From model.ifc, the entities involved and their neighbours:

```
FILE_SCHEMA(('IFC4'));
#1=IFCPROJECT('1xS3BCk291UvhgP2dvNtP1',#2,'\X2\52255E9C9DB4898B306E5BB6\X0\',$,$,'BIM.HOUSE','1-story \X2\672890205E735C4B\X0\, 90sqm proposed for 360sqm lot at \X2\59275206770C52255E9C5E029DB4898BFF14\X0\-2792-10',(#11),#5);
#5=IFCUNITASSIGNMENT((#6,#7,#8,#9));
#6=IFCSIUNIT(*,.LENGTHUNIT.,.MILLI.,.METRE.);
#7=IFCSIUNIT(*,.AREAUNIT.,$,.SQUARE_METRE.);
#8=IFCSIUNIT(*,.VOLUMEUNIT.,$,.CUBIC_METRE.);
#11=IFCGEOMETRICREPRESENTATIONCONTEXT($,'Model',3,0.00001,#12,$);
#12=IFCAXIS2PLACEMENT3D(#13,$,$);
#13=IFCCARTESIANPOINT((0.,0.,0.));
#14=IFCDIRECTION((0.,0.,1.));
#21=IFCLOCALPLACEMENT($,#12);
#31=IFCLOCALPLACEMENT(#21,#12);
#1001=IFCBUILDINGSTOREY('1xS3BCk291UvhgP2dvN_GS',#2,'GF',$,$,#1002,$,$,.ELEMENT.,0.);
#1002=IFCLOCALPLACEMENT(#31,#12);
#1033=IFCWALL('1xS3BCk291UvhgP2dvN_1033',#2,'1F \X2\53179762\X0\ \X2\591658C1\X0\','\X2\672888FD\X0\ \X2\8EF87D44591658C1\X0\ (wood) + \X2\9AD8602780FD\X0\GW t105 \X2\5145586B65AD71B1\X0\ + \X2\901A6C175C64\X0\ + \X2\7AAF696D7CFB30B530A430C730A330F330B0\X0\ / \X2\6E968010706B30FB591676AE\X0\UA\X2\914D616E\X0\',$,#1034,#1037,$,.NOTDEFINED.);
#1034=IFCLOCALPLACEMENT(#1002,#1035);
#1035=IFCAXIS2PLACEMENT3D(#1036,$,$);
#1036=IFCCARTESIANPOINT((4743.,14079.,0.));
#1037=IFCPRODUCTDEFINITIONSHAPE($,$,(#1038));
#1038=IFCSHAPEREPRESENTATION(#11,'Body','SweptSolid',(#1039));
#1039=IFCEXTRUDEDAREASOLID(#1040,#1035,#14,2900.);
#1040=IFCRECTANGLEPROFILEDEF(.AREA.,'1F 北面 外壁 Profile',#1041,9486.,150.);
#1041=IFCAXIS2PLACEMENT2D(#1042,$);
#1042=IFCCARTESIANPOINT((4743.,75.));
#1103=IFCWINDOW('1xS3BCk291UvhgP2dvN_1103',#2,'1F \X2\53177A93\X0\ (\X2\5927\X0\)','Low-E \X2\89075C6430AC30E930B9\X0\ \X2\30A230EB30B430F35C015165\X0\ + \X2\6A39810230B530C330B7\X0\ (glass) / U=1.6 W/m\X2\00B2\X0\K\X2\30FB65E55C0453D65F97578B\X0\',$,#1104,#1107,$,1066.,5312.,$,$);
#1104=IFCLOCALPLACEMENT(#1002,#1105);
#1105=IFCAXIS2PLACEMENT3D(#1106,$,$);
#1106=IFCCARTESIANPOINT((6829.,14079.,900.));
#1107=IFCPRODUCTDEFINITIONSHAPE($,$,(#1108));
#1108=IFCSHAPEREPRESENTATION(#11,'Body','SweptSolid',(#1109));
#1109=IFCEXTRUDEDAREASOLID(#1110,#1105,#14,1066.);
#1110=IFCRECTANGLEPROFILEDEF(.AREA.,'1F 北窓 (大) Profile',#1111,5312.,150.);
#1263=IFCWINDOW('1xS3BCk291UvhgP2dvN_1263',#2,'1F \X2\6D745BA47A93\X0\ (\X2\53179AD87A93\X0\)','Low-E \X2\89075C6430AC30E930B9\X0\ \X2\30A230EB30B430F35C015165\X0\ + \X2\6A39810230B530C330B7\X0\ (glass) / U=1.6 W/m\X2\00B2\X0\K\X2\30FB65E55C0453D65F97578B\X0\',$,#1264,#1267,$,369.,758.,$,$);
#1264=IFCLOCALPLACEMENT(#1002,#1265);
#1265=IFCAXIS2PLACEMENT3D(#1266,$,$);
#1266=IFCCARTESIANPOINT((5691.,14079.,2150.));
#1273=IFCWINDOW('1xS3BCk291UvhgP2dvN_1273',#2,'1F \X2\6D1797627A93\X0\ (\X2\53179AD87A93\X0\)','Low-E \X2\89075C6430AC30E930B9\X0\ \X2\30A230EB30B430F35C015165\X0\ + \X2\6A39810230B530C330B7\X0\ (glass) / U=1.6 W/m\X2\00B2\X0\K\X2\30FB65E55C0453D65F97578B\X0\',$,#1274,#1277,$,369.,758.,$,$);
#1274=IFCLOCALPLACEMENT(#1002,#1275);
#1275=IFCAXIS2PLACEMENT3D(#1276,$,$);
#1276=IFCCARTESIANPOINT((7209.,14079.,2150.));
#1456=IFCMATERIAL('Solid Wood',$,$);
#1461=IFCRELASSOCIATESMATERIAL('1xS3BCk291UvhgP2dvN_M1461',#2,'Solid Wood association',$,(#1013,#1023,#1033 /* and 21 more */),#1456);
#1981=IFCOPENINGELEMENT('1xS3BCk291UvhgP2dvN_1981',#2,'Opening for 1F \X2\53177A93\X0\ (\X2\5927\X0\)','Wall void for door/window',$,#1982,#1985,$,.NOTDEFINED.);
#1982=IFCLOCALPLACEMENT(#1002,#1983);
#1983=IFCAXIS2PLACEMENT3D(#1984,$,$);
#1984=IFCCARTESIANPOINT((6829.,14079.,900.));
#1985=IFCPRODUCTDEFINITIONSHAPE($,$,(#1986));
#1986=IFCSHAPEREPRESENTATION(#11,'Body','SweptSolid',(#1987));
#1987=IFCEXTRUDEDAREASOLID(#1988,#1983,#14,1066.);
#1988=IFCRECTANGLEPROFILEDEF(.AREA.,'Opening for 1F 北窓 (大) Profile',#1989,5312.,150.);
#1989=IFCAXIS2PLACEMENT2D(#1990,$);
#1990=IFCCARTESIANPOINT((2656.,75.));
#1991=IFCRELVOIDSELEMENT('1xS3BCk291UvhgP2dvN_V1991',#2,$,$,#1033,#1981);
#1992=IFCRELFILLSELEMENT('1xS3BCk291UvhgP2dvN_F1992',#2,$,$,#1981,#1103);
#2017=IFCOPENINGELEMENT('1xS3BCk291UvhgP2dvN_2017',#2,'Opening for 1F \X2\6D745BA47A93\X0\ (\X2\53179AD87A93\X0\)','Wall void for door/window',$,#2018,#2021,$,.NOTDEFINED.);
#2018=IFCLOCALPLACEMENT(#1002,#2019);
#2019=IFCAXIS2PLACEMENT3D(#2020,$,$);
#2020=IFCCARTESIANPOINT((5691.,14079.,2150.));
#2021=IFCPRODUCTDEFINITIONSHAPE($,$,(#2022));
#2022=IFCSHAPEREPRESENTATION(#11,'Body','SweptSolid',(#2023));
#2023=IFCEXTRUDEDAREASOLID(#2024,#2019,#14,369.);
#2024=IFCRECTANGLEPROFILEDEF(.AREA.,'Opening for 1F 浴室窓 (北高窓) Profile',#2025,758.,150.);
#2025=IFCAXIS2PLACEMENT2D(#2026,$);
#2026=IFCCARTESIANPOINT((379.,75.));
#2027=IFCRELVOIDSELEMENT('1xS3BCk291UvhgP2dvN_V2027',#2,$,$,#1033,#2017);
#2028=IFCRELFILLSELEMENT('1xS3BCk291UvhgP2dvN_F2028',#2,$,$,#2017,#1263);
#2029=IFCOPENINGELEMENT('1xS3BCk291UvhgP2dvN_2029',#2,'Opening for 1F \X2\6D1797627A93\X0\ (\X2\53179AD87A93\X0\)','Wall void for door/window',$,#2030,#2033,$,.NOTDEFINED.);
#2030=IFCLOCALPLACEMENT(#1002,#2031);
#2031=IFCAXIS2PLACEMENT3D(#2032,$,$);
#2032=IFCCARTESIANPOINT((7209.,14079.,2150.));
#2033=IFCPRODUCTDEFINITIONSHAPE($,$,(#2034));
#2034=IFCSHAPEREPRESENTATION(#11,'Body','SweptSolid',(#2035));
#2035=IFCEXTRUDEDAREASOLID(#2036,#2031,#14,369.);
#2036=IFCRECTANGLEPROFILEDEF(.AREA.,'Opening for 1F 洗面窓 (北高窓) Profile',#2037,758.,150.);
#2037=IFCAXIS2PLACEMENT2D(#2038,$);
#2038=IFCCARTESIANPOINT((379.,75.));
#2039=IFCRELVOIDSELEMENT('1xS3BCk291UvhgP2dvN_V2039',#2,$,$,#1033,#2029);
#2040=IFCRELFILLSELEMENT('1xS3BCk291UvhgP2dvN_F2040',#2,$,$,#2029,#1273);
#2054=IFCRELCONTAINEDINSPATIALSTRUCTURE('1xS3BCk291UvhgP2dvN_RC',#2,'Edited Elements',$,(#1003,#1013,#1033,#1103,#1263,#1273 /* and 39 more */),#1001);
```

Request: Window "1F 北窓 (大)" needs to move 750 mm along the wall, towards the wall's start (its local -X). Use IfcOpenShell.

```python
import ifcopenshell
import ifcopenshell.api.geometry
import ifcopenshell.util.placement
import ifcopenshell.util.unit

model = ifcopenshell.open("model.ifc")
unit_scale = ifcopenshell.util.unit.calculate_unit_scale(model)

window = model.by_id(1103)
opening = window.FillsVoids[0].RelatingOpeningElement
wall = opening.VoidsElements[0].RelatingBuildingElement

wall_matrix = ifcopenshell.util.placement.get_local_placement(wall.ObjectPlacement)
shift = wall_matrix[:3, 0] * -0.75 / unit_scale
before = ifcopenshell.util.placement.get_local_placement(window.ObjectPlacement)[:3, 3].copy()

# The window is not placed relative to its opening, so move both.
for product in (opening, window):
    matrix = ifcopenshell.util.placement.get_local_placement(product.ObjectPlacement)
    matrix[:3, 3] += shift
    ifcopenshell.api.geometry.edit_object_placement(model, product=product, matrix=matrix, is_si=False)

after = ifcopenshell.util.placement.get_local_placement(window.ObjectPlacement)[:3, 3]
print("window moved by", (after - before).round(3) + 0.0)

model.write("model_v2.ifc")
```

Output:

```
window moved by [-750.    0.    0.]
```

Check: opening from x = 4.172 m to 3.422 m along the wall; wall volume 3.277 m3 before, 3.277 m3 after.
